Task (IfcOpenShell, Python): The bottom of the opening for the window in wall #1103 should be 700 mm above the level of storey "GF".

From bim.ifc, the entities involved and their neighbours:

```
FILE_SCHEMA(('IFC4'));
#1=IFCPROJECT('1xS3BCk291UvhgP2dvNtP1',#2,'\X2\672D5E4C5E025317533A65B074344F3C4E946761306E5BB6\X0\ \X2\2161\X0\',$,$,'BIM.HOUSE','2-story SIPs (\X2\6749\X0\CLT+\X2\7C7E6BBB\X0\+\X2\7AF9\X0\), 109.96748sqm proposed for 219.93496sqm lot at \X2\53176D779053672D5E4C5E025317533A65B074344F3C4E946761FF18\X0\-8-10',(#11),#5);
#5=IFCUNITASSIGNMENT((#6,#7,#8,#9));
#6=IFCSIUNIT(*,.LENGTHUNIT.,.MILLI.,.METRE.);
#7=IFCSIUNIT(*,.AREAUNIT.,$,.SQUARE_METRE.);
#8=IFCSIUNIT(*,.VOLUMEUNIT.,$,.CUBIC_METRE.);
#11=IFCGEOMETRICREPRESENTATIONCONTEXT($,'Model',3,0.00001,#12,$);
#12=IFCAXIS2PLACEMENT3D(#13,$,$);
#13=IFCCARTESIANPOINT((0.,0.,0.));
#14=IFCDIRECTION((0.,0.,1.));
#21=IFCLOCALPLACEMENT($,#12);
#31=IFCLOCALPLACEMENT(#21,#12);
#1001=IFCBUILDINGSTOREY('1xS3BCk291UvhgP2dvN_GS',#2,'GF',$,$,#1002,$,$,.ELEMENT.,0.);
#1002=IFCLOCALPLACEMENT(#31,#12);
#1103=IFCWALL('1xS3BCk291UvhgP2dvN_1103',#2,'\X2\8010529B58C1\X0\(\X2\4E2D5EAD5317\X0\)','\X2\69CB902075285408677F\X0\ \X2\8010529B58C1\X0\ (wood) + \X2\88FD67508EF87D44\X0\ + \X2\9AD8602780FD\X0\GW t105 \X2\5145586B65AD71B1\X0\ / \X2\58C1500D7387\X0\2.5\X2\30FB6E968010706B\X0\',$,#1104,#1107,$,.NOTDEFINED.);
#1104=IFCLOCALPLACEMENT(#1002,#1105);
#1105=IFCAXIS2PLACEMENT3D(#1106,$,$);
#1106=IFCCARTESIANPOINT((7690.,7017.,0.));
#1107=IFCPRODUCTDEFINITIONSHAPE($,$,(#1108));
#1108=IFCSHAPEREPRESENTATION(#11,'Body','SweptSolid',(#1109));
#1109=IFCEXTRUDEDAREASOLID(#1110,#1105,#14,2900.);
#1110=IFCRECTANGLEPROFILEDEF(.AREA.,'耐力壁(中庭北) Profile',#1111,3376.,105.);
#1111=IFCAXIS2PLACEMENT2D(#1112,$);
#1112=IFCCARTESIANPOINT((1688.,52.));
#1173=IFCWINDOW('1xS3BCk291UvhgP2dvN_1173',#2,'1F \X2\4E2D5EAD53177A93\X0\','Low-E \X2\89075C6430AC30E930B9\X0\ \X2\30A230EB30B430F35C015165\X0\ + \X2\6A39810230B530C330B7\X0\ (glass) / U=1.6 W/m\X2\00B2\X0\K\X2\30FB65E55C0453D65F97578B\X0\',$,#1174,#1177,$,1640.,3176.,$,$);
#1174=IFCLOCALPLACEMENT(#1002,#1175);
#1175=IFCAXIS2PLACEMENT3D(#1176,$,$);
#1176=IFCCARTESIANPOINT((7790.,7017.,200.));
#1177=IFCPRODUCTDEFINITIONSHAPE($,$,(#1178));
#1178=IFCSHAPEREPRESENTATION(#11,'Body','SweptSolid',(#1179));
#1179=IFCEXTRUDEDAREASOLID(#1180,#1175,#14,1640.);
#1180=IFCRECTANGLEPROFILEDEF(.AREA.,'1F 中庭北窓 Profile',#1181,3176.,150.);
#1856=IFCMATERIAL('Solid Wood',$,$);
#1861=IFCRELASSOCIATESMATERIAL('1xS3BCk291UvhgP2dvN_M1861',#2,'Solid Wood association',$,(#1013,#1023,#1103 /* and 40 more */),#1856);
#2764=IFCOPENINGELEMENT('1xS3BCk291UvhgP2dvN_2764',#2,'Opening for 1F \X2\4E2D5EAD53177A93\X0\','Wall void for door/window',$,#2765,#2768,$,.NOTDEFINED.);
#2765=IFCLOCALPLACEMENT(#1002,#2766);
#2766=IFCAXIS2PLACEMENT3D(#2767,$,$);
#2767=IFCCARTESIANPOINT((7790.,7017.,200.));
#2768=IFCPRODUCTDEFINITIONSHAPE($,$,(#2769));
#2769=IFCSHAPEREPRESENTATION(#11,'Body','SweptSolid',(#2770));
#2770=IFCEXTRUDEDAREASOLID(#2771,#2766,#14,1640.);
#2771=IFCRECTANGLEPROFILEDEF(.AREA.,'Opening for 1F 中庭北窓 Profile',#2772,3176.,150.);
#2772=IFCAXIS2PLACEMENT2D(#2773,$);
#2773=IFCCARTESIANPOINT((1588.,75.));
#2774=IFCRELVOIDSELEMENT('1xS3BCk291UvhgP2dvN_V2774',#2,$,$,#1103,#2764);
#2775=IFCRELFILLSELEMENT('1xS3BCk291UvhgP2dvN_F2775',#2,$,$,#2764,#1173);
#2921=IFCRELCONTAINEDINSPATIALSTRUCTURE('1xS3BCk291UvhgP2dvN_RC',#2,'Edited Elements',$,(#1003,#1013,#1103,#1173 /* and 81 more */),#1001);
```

```python
import numpy as np
import ifcopenshell
import ifcopenshell.api.geometry
import ifcopenshell.geom
import ifcopenshell.util.element
import ifcopenshell.util.placement
import ifcopenshell.util.shape
import ifcopenshell.util.unit

model = ifcopenshell.open("bim.ifc")
unit_scale = ifcopenshell.util.unit.calculate_unit_scale(model)

window = model.by_id(1173)
opening = window.FillsVoids[0].RelatingOpeningElement
storey = ifcopenshell.util.element.get_container(window, ifc_class="IfcBuildingStorey")
level = ifcopenshell.util.placement.get_local_placement(storey.ObjectPlacement)[2, 3]

# The opening's origin need not be at the sill, so measure its lowest point.
shape = ifcopenshell.geom.create_shape(ifcopenshell.geom.settings(), opening)
bottom = ifcopenshell.util.shape.get_shape_bottom_elevation(shape, shape.geometry) / unit_scale
dz = level + 700.0 - bottom

shift = np.array([0.0, 0.0, dz])
# The window is not placed relative to its opening, so move both.
for product in (opening, window):
    matrix = ifcopenshell.util.placement.get_local_placement(product.ObjectPlacement)
    matrix[:3, 3] += shift
    ifcopenshell.api.geometry.edit_object_placement(model, product=product, matrix=matrix, is_si=False)

print(f"moved by {dz * unit_scale:+.3f} m")

model.write("bim-out.ifc")
```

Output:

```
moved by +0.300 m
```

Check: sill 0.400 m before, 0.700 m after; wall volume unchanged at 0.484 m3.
